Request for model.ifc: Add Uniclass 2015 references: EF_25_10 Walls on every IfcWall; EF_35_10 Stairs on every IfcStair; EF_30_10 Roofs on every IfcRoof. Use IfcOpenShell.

First a look at what the model holds.

```python
import ifcopenshell

model = ifcopenshell.open("model.ifc")
print(model.schema)
print("classifications:", [c.Name for c in model.by_type("IfcClassification")])
for ifc_class in ("IfcDoor", "IfcRoof", "IfcStair", "IfcWall", "IfcWindow"):
    print(ifc_class, len(model.by_type(ifc_class)))
```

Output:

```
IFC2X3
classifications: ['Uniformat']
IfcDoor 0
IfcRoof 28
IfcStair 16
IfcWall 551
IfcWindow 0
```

```python
import ifcopenshell
import ifcopenshell.api.classification

model = ifcopenshell.open("model.ifc")

# IFC2X3 requires Source and Edition and has no link from the project to the system.
system = model.create_entity("IfcClassification", Source="NBS", Edition="2015", Name="Uniclass 2015")

codes = {
    "IfcWall": ("EF_25_10", "Walls"),
    "IfcStair": ("EF_35_10", "Stairs"),
    "IfcRoof": ("EF_30_10", "Roofs"),
}
for ifc_class, (code, name) in codes.items():
    products = model.by_type(ifc_class)
    ifcopenshell.api.classification.add_reference(
        model, products=products, classification=system, identification=code, name=name
    )
    print(code, len(products))

model.write("model_edited.ifc")
```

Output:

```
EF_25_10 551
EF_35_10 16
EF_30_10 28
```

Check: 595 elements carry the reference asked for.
